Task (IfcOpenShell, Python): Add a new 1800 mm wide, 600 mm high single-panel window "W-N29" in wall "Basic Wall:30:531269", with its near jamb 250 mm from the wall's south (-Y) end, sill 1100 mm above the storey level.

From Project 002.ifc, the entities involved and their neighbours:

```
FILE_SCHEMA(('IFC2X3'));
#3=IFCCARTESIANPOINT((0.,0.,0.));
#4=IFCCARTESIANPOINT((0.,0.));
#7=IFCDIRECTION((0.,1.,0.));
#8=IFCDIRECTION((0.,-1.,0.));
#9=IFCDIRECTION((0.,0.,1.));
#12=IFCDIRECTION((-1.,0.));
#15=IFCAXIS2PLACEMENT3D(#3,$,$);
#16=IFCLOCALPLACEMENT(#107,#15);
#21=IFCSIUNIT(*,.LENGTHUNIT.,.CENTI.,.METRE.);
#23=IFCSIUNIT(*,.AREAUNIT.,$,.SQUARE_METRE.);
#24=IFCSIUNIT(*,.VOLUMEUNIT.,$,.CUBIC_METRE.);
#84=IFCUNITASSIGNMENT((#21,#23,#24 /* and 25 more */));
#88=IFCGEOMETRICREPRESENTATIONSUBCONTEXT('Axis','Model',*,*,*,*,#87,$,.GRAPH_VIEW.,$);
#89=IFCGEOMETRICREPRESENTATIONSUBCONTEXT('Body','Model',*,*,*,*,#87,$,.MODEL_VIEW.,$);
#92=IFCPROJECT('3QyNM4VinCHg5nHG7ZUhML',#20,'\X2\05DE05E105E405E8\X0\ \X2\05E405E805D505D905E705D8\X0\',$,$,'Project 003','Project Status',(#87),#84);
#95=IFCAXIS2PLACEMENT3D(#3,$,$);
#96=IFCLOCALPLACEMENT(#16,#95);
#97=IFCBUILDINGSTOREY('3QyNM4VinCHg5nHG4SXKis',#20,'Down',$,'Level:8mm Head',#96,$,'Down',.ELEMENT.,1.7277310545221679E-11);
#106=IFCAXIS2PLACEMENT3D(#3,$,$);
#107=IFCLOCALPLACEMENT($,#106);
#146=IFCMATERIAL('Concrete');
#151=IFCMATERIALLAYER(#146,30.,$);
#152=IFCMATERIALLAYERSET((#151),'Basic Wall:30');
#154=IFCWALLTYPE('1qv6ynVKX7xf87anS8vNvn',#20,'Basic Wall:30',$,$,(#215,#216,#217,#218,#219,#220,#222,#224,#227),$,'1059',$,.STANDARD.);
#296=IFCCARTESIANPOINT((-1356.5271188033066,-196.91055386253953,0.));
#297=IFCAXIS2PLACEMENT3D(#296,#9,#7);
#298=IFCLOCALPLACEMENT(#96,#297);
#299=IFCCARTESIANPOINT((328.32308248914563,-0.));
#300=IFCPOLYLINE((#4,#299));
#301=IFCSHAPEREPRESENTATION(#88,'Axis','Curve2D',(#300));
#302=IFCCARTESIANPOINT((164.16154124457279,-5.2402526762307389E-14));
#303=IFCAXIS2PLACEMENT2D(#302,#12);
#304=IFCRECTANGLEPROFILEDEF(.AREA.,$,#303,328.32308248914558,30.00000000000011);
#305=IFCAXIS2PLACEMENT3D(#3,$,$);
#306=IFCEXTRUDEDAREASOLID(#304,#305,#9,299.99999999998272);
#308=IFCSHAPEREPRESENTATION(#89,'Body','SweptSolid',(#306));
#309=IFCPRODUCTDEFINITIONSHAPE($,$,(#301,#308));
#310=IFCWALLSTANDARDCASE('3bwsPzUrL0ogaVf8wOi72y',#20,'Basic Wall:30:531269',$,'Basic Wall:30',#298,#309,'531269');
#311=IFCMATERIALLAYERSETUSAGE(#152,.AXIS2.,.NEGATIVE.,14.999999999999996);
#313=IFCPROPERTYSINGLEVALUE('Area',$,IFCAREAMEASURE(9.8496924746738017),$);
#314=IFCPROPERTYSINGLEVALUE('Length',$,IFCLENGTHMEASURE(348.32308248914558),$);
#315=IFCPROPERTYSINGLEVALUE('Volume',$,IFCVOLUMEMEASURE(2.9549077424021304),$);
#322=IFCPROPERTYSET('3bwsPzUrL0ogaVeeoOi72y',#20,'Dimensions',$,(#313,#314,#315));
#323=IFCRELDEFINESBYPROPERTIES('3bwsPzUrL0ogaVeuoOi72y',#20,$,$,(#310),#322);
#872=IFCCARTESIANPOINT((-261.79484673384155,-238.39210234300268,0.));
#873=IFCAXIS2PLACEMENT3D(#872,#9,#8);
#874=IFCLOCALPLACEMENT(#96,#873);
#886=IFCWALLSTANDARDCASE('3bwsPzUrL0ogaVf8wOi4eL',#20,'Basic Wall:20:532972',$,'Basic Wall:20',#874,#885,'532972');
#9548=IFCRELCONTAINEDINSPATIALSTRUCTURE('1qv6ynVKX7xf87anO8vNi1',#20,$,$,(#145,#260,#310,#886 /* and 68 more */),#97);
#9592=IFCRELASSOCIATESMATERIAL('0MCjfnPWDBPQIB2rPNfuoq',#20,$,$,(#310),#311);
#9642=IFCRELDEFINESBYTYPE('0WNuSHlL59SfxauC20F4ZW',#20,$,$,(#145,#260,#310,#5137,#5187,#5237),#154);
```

```python
import numpy as np
import ifcopenshell
import ifcopenshell.api.feature
import ifcopenshell.api.geometry
import ifcopenshell.api.pset
import ifcopenshell.api.root
import ifcopenshell.api.spatial
import ifcopenshell.api.type
import ifcopenshell.geom
import ifcopenshell.util.element
import ifcopenshell.util.placement
import ifcopenshell.util.representation
import ifcopenshell.util.shape
import ifcopenshell.util.unit

model = ifcopenshell.open("Project 002.ifc")
unit_scale = ifcopenshell.util.unit.calculate_unit_scale(model)
area_scale = ifcopenshell.util.unit.calculate_unit_scale(model, "AREAUNIT")
volume_scale = ifcopenshell.util.unit.calculate_unit_scale(model, "VOLUMEUNIT")
settings = ifcopenshell.geom.settings()


def volume(element):
    """Net volume in cubic metres, openings subtracted."""
    shape = ifcopenshell.geom.create_shape(settings, element)
    return ifcopenshell.util.shape.get_volume(shape.geometry)


wall = model.by_id(310)
storey = ifcopenshell.util.element.get_container(wall, ifc_class="IfcBuildingStorey")
context = ifcopenshell.util.representation.get_context(model, "Model", "Body", "MODEL_VIEW")
before = volume(wall)

width, height, from_end, sill = 1.8, 0.6, 0.25, 1.1  # metres

# The wall runs along its own X axis, and the end named is its -X end.
wall_shape = ifcopenshell.geom.create_shape(settings, wall)
x, y, z = ifcopenshell.util.shape.get_vertices(wall_shape.geometry).T
start = x.min() + from_end
face, thickness = float(y.min()), float(y.max() - y.min())
wall_matrix = ifcopenshell.util.placement.get_local_placement(wall.ObjectPlacement)
level = ifcopenshell.util.placement.get_local_placement(storey.ObjectPlacement)[2, 3]


def in_wall(x, y):
    """Placement at x, y metres in the wall's axes, at sill height."""
    matrix = wall_matrix.copy()
    matrix[:, 3] = wall_matrix @ np.array([x / unit_scale, y / unit_scale, 0.0, 1.0])
    matrix[2, 3] = level + sill / unit_scale
    return matrix


# Opening: a box that overshoots both wall faces by 50 mm.
opening = ifcopenshell.api.root.create_entity(model, ifc_class="IfcOpeningElement")
box = ifcopenshell.api.geometry.add_wall_representation(
    model, context=context, length=width, height=height, thickness=thickness + 0.1
)
ifcopenshell.api.geometry.assign_representation(model, product=opening, representation=box)
ifcopenshell.api.geometry.edit_object_placement(model, product=opening, matrix=in_wall(start, face - 0.05), is_si=False)
ifcopenshell.api.feature.add_feature(model, feature=opening, element=wall)

window = ifcopenshell.api.root.create_entity(model, ifc_class="IfcWindow", name="W-N29")
window.OverallWidth, window.OverallHeight = width / unit_scale, height / unit_scale
body = ifcopenshell.api.geometry.add_window_representation(
    model,
    context=context,
    overall_width=window.OverallWidth,
    overall_height=window.OverallHeight,
    partition_type="SINGLE_PANEL",
)
ifcopenshell.api.geometry.assign_representation(model, product=window, representation=body)
ifcopenshell.api.spatial.assign_container(model, products=[window], relating_structure=storey)
fills = ifcopenshell.api.feature.add_filling(model, opening=opening, element=window)
fills.OwnerHistory = window.OwnerHistory  # required in IFC2X3

# IFC2X3 keeps the operation on the window style.
style = ifcopenshell.api.root.create_entity(model, ifc_class="IfcWindowStyle", name="W-N29")
style.OperationType, style.ConstructionType = "SINGLE_PANEL", "NOTDEFINED"
style.ParameterTakesPrecedence = style.Sizeable = False
ifcopenshell.api.type.assign_type(model, related_objects=[window], relating_type=style)

# Centre the window in the wall's thickness.
ifcopenshell.api.geometry.edit_object_placement(model, product=window, matrix=in_wall(start, face), is_si=False)
window_shape = ifcopenshell.geom.create_shape(settings, window)
depth = ifcopenshell.util.shape.get_vertices(window_shape.geometry)[:, 1]
offset = face + thickness / 2 - (depth.min() + depth.max()) / 2
ifcopenshell.api.geometry.edit_object_placement(model, product=window, matrix=in_wall(start, offset), is_si=False)

after = volume(wall)

# Update the wall's stored quantities.
pset = model.by_id(ifcopenshell.util.element.get_pset(wall, "Dimensions", should_inherit=False)["id"])
ifcopenshell.api.pset.edit_pset(model, pset=pset, properties={
    "Area": model.create_entity("IfcAreaMeasure", after / thickness / area_scale),
    "Volume": model.create_entity("IfcVolumeMeasure", after / volume_scale),
})

print(f"wall volume {before:.3f} -> {after:.3f} m3")

model.write("Project 002_rev.ifc")
```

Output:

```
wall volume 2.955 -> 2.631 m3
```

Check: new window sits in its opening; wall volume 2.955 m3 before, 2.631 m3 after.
